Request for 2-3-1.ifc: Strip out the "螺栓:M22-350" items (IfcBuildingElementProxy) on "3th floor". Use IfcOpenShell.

First a look at what the model holds.

```python
import ifcopenshell
import ifcopenshell.util.element

model = ifcopenshell.open("2-3-1.ifc")
print(model.schema)
storey = next(s for s in model.by_type("IfcBuildingStorey") if s.Name == "3th floor")
proxies = [e for e in ifcopenshell.util.element.get_decomposition(storey) if e.is_a("IfcBuildingElementProxy")]
seen = {}
for e in proxies:
    element_type = ifcopenshell.util.element.get_type(e)
    name = element_type.Name if element_type not in (None, e) else None
    seen[name] = seen.get(name, 0) + 1
for name, count in sorted(seen.items(), key=str):
    print(count, "x", name)
```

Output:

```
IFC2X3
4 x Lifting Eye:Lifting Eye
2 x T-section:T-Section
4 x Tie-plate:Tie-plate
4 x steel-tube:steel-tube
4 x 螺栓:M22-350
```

```python
import ifcopenshell
import ifcopenshell.api.root
import ifcopenshell.util.element

model = ifcopenshell.open("2-3-1.ifc")

storey = next(s for s in model.by_type("IfcBuildingStorey") if s.Name == "3th floor")
proxies = [e for e in ifcopenshell.util.element.get_decomposition(storey) if e.is_a("IfcBuildingElementProxy")]
targets = [e for e in proxies if (t := ifcopenshell.util.element.get_type(e)) not in (None, e) and t.Name == "螺栓:M22-350"]

for e in targets:
    ifcopenshell.api.root.remove_product(model, product=e)
print(len(targets), "removed")

model.write("2-3-1_edited.ifc")
```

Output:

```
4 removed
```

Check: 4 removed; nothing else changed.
